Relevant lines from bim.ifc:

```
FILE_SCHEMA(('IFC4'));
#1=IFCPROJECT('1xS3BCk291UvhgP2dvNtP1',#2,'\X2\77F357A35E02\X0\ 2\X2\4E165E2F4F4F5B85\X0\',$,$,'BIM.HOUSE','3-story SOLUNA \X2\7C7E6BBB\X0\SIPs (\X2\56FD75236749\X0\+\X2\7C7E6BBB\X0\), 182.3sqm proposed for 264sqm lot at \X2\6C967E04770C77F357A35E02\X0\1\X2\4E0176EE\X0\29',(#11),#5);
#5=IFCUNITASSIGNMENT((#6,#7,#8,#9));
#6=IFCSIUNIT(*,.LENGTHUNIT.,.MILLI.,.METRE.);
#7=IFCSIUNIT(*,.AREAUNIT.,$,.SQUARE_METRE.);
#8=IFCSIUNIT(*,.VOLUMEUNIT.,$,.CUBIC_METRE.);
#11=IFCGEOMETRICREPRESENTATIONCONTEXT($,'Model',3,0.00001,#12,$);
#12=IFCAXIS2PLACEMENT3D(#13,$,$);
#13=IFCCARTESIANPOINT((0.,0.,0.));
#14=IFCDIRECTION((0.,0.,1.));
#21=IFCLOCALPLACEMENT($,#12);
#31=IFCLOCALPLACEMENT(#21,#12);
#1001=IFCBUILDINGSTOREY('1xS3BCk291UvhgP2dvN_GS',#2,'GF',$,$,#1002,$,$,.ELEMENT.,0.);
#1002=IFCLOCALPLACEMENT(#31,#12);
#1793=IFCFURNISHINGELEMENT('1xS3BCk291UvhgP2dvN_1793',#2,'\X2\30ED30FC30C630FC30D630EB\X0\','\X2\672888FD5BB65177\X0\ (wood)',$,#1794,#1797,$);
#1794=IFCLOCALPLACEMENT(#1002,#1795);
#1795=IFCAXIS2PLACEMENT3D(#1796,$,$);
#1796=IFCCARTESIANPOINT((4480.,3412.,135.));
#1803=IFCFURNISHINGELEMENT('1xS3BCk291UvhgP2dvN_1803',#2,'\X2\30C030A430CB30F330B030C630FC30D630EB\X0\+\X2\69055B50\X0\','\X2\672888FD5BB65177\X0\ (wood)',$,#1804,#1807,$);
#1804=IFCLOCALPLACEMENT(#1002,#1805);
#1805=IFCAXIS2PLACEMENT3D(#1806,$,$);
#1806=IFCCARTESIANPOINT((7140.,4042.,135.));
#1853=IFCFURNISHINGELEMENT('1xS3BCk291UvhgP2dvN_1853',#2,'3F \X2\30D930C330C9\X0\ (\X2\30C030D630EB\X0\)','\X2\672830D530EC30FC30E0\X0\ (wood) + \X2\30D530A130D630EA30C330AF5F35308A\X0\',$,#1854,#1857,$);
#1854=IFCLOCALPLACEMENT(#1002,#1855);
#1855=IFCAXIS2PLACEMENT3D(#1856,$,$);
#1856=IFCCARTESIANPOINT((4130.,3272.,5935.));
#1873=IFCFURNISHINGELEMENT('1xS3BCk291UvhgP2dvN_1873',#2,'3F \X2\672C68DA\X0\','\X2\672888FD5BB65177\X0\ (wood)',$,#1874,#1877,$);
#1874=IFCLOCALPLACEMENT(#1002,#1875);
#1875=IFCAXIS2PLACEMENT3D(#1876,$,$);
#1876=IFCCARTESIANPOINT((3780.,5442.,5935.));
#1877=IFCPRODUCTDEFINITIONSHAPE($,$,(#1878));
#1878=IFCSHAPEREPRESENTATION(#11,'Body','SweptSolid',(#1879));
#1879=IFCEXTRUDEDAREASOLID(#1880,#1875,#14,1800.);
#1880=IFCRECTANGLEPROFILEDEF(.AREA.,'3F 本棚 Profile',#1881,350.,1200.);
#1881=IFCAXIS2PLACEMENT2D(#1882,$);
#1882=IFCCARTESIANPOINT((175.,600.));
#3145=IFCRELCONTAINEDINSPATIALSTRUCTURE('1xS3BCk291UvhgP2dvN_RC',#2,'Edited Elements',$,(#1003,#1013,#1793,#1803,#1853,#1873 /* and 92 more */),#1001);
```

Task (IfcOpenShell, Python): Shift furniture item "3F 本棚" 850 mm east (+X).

```python
import ifcopenshell
import ifcopenshell.api.geometry
import ifcopenshell.util.placement
import ifcopenshell.util.unit

model = ifcopenshell.open("bim.ifc")
unit_scale = ifcopenshell.util.unit.calculate_unit_scale(model)

item = model.by_guid("1xS3BCk291UvhgP2dvN_1873")
matrix = ifcopenshell.util.placement.get_local_placement(item.ObjectPlacement)
matrix[0, 3] += 0.85 / unit_scale
ifcopenshell.api.geometry.edit_object_placement(model, product=item, matrix=matrix, is_si=False)

print(ifcopenshell.util.placement.get_local_placement(item.ObjectPlacement).round(3) + 0.0)

model.write("bim_rev.ifc")
```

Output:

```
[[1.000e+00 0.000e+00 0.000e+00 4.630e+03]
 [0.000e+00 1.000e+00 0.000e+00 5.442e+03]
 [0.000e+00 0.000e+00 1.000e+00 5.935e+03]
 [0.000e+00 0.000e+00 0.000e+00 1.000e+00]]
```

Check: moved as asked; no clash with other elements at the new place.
